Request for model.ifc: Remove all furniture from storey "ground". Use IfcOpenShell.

First a look at what the model holds.

```python
import ifcopenshell
import ifcopenshell.util.element

model = ifcopenshell.open("model.ifc")
print(model.schema)
storey = next(s for s in model.by_type("IfcBuildingStorey") if s.Name == "ground")
furniture = [e for e in ifcopenshell.util.element.get_decomposition(storey) if e.is_a("IfcFurnishingElement")]
seen = {}
for e in furniture:
    element_type = ifcopenshell.util.element.get_type(e)
    name = element_type.Name if element_type not in (None, e) else None
    seen[name] = seen.get(name, 0) + 1
for name, count in sorted(seen.items(), key=str):
    print(count, "x", name)
```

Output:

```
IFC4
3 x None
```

```python
import ifcopenshell
import ifcopenshell.api.root
import ifcopenshell.util.element

model = ifcopenshell.open("model.ifc")

storey = next(s for s in model.by_type("IfcBuildingStorey") if s.Name == "ground")
furniture = [e for e in ifcopenshell.util.element.get_decomposition(storey) if e.is_a("IfcFurnishingElement")]

for e in furniture:
    ifcopenshell.api.root.remove_product(model, product=e)
print(len(furniture), "removed")

model.write("model_edited.ifc")
```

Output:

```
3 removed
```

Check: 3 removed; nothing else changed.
